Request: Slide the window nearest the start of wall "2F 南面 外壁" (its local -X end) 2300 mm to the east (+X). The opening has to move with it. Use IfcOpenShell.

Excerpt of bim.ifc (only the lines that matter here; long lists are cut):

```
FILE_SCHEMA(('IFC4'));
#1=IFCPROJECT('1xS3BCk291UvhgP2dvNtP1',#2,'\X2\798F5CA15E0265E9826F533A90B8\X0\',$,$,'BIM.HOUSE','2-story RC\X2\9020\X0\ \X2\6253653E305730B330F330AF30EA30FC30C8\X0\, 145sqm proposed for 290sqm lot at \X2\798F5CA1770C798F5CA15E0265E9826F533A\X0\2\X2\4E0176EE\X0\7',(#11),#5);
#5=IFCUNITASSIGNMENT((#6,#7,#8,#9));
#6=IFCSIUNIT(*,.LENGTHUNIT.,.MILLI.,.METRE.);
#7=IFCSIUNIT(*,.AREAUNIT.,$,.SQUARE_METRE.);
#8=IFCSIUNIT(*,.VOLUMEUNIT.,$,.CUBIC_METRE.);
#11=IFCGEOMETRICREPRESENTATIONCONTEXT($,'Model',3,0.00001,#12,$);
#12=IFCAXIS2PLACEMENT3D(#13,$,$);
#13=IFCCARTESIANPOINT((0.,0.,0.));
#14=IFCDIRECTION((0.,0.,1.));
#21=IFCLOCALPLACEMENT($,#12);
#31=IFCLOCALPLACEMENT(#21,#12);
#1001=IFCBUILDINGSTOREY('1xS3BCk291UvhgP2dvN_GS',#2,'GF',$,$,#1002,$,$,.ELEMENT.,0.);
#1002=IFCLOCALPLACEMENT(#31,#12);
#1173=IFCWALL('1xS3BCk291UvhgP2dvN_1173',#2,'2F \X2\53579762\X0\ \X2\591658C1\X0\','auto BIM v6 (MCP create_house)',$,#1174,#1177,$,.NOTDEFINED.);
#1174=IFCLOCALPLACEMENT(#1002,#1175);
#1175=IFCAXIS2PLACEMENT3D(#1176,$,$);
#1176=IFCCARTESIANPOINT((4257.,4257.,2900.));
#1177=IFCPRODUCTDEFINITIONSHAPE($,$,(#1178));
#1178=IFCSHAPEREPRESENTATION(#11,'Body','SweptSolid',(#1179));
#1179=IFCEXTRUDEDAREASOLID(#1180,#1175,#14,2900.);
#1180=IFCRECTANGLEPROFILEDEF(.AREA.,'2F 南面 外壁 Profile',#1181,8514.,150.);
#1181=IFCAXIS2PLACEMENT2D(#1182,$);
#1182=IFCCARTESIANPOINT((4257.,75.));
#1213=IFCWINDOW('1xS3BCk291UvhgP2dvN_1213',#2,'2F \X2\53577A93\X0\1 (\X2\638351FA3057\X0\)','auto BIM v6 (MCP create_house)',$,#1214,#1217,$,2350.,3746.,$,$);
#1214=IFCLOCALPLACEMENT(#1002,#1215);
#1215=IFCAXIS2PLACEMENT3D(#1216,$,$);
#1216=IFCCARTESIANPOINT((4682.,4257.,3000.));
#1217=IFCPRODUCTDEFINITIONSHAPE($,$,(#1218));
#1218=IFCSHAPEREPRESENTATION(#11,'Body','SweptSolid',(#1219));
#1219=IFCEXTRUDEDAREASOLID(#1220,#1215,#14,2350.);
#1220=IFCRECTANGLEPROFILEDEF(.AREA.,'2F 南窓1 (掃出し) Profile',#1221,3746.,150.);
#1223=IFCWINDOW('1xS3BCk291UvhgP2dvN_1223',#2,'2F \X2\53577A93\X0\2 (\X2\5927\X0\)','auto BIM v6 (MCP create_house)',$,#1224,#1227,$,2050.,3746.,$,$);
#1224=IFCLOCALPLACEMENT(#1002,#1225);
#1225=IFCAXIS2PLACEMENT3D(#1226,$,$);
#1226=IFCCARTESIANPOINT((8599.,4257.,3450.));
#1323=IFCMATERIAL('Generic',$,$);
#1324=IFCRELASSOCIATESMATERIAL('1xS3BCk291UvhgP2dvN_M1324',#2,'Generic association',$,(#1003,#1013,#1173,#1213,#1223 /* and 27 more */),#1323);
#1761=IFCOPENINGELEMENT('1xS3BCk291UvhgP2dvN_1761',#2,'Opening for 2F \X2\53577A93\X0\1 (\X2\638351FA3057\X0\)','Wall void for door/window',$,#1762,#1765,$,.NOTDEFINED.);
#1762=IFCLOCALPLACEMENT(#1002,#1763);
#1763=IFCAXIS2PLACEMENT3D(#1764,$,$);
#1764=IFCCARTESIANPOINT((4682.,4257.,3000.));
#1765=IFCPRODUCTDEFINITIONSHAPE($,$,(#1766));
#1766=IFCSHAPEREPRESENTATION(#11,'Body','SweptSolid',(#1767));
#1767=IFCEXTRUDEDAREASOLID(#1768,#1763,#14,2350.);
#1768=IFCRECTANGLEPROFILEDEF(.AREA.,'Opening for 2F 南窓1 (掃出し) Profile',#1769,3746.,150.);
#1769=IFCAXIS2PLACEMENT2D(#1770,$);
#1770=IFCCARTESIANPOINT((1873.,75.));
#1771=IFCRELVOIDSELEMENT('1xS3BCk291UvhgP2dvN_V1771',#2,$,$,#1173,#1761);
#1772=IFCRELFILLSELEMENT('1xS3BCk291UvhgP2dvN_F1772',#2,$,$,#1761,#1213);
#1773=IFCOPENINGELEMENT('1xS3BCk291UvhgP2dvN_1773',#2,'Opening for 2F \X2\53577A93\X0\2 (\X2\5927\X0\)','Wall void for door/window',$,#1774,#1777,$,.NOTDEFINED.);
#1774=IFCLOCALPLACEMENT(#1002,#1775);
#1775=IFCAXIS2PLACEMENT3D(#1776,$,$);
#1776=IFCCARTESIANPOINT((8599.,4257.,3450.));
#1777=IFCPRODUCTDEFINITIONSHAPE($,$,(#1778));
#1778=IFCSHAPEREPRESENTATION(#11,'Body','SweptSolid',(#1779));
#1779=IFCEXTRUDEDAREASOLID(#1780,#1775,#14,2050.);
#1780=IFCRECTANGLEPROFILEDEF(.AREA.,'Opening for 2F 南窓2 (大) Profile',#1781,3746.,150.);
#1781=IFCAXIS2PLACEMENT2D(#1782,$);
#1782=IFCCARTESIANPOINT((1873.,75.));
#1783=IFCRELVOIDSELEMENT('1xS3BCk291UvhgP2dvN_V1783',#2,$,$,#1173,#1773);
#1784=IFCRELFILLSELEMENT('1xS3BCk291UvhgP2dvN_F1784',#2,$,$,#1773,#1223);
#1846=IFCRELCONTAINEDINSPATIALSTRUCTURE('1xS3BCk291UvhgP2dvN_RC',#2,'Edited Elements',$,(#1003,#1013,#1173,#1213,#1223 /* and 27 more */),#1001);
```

```python
import ifcopenshell
import ifcopenshell.api.geometry
import ifcopenshell.util.placement

model = ifcopenshell.open("bim.ifc")

window = model.by_guid("1xS3BCk291UvhgP2dvN_1213")
opening = window.FillsVoids[0].RelatingOpeningElement
wall = opening.VoidsElements[0].RelatingBuildingElement

wall_matrix = ifcopenshell.util.placement.get_local_placement(wall.ObjectPlacement)
shift = wall_matrix[:3, 0] * 2300.0
before = ifcopenshell.util.placement.get_local_placement(window.ObjectPlacement)[:3, 3].copy()

# The window is not placed relative to its opening, so move both.
for product in (opening, window):
    matrix = ifcopenshell.util.placement.get_local_placement(product.ObjectPlacement)
    matrix[:3, 3] += shift
    ifcopenshell.api.geometry.edit_object_placement(model, product=product, matrix=matrix, is_si=False)

after = ifcopenshell.util.placement.get_local_placement(window.ObjectPlacement)[:3, 3]
print("window moved by", (after - before).round(3) + 0.0)

model.write("bim_rev.ifc")
```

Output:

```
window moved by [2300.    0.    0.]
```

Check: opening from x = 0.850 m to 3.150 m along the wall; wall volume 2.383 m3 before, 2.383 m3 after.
